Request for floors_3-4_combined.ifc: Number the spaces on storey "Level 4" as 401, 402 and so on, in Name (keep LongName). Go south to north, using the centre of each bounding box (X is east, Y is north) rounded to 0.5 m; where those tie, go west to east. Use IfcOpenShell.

First a look at what the model holds.

```python
import ifcopenshell
import ifcopenshell.util.element
import ifcopenshell.util.placement

model = ifcopenshell.open("floors_3-4_combined.ifc")
print(model.schema)
storey = next(s for s in model.by_type("IfcBuildingStorey") if s.Name == "Level 4")
spaces = [e for e in ifcopenshell.util.element.get_decomposition(storey) if e.is_a("IfcSpace")]
for e in sorted(spaces, key=lambda e: e.id()):
    origin = ifcopenshell.util.placement.get_local_placement(e.ObjectPlacement)[:3, 3]
    print(e.id(), e.Name, e.LongName, origin.round(2) + 0.0, sep=" | ")
```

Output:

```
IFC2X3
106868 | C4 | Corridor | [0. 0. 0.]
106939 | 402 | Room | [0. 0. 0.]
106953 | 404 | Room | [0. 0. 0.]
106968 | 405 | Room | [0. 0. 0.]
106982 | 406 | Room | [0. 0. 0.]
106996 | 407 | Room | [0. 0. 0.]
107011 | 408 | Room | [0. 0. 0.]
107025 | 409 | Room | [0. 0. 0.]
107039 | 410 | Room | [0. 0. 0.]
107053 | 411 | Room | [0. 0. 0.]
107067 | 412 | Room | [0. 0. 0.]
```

```python
import ifcopenshell
import ifcopenshell.geom
import ifcopenshell.util.element
import ifcopenshell.util.shape

model = ifcopenshell.open("floors_3-4_combined.ifc")
settings = ifcopenshell.geom.settings()
settings.set("use-world-coords", True)


def centre(element):
    shape = ifcopenshell.geom.create_shape(settings, element)
    return ifcopenshell.util.shape.get_bbox_centroid(shape.geometry)


storey = next(s for s in model.by_type("IfcBuildingStorey") if s.Name == "Level 4")
spaces = [e for e in ifcopenshell.util.element.get_decomposition(storey) if e.is_a("IfcSpace")]

# Insertion points can sit at a corner or the storey origin, so sort by the geometry (in metres).
centres = {e: centre(e) for e in spaces}
spaces.sort(key=lambda e: (round(centres[e][1] / 0.5), centres[e][0]))

for i, e in enumerate(spaces, start=1):
    number = f"4{i:02d}"
    e.Name = number
    print(e.id(), number)

model.write("floors_3-4_combined_rev.ifc")
```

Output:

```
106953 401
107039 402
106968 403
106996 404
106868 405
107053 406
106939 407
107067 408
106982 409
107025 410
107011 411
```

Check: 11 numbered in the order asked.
